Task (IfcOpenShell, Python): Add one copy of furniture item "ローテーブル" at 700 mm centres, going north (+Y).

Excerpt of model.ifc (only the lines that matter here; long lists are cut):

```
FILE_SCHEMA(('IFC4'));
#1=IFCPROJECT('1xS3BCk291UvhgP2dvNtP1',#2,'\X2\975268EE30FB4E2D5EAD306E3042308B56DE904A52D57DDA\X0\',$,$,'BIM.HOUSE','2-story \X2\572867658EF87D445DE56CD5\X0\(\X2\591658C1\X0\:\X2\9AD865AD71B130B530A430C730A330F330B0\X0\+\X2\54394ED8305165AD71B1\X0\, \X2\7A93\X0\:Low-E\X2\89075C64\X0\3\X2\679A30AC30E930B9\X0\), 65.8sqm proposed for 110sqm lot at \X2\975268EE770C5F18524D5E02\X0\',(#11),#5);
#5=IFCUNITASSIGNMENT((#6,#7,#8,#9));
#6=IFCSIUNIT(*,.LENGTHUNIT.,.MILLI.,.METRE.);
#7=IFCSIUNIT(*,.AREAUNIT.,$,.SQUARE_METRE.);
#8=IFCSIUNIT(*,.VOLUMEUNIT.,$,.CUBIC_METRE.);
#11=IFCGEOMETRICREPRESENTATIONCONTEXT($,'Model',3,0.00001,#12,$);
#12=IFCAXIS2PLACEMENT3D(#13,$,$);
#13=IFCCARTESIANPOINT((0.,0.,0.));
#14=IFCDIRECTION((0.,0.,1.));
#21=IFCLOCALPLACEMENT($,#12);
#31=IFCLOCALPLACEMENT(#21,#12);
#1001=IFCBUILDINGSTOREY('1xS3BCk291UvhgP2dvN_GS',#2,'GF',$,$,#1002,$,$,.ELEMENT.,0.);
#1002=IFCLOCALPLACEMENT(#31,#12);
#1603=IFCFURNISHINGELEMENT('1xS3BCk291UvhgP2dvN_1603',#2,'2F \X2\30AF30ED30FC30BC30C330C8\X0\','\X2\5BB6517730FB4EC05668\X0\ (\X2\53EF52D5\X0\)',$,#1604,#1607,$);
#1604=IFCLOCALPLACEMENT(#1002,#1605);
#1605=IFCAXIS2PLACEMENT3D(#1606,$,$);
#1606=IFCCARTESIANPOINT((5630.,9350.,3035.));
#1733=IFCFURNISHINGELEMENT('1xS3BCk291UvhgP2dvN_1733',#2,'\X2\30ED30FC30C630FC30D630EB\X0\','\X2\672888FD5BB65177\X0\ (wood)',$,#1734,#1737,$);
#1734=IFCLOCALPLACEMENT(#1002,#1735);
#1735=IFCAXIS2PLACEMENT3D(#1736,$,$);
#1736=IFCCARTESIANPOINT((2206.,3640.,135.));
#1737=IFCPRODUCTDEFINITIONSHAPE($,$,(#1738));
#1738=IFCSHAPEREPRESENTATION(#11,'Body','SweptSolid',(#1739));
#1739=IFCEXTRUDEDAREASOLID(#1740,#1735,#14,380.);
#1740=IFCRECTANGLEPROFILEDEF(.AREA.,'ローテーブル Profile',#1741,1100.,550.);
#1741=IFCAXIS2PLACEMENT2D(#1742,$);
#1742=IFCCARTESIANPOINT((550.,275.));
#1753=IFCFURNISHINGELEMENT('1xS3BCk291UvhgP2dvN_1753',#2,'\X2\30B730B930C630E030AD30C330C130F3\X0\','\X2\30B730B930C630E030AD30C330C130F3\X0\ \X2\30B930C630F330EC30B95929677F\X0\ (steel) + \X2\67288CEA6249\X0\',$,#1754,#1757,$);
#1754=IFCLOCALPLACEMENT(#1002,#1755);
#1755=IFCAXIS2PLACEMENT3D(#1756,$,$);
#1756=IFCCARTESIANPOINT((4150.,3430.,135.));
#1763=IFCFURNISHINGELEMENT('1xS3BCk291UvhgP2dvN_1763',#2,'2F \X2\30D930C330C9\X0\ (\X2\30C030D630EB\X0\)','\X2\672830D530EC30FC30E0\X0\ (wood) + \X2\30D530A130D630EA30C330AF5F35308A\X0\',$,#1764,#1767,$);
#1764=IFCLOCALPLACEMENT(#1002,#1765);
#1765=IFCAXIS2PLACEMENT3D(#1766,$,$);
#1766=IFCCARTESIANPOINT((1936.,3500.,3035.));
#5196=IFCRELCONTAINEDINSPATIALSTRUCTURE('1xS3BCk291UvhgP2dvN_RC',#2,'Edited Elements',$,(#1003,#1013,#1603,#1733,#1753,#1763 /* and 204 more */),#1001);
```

```python
import numpy as np
import ifcopenshell
import ifcopenshell.api.geometry
import ifcopenshell.api.root
import ifcopenshell.util.element
import ifcopenshell.util.placement

model = ifcopenshell.open("model.ifc")


def reuse_history(source, copy):
    """copy_class also copies each property set's owner history, people and application; keep the originals."""
    for rel in copy.IsDefinedBy:
        if rel.is_a("IfcRelDefinesByProperties") and (history := rel.RelatingPropertyDefinition.OwnerHistory):
            rel.RelatingPropertyDefinition.OwnerHistory = source.OwnerHistory
            ifcopenshell.util.element.remove_deep2(model, history)


source = model.by_guid("1xS3BCk291UvhgP2dvN_1733")
base = ifcopenshell.util.placement.get_local_placement(source.ObjectPlacement)
step = np.array([0.0, 1.0, 0.0]) * 700.0

for i in range(1, 2):
    copy = ifcopenshell.api.root.copy_class(model, product=source)
    copy.Representation = ifcopenshell.util.element.copy_deep(
        model, source.Representation, exclude=["IfcGeometricRepresentationContext", "IfcRepresentationMap"]
    )
    reuse_history(source, copy)
    matrix = base.copy()
    matrix[:3, 3] += i * step
    print("added at", matrix[:3, 3].round(3) + 0.0)
    ifcopenshell.api.geometry.edit_object_placement(model, product=copy, matrix=matrix, is_si=False)

model.write("model_updated.ifc")
```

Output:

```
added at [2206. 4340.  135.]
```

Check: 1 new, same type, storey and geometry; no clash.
